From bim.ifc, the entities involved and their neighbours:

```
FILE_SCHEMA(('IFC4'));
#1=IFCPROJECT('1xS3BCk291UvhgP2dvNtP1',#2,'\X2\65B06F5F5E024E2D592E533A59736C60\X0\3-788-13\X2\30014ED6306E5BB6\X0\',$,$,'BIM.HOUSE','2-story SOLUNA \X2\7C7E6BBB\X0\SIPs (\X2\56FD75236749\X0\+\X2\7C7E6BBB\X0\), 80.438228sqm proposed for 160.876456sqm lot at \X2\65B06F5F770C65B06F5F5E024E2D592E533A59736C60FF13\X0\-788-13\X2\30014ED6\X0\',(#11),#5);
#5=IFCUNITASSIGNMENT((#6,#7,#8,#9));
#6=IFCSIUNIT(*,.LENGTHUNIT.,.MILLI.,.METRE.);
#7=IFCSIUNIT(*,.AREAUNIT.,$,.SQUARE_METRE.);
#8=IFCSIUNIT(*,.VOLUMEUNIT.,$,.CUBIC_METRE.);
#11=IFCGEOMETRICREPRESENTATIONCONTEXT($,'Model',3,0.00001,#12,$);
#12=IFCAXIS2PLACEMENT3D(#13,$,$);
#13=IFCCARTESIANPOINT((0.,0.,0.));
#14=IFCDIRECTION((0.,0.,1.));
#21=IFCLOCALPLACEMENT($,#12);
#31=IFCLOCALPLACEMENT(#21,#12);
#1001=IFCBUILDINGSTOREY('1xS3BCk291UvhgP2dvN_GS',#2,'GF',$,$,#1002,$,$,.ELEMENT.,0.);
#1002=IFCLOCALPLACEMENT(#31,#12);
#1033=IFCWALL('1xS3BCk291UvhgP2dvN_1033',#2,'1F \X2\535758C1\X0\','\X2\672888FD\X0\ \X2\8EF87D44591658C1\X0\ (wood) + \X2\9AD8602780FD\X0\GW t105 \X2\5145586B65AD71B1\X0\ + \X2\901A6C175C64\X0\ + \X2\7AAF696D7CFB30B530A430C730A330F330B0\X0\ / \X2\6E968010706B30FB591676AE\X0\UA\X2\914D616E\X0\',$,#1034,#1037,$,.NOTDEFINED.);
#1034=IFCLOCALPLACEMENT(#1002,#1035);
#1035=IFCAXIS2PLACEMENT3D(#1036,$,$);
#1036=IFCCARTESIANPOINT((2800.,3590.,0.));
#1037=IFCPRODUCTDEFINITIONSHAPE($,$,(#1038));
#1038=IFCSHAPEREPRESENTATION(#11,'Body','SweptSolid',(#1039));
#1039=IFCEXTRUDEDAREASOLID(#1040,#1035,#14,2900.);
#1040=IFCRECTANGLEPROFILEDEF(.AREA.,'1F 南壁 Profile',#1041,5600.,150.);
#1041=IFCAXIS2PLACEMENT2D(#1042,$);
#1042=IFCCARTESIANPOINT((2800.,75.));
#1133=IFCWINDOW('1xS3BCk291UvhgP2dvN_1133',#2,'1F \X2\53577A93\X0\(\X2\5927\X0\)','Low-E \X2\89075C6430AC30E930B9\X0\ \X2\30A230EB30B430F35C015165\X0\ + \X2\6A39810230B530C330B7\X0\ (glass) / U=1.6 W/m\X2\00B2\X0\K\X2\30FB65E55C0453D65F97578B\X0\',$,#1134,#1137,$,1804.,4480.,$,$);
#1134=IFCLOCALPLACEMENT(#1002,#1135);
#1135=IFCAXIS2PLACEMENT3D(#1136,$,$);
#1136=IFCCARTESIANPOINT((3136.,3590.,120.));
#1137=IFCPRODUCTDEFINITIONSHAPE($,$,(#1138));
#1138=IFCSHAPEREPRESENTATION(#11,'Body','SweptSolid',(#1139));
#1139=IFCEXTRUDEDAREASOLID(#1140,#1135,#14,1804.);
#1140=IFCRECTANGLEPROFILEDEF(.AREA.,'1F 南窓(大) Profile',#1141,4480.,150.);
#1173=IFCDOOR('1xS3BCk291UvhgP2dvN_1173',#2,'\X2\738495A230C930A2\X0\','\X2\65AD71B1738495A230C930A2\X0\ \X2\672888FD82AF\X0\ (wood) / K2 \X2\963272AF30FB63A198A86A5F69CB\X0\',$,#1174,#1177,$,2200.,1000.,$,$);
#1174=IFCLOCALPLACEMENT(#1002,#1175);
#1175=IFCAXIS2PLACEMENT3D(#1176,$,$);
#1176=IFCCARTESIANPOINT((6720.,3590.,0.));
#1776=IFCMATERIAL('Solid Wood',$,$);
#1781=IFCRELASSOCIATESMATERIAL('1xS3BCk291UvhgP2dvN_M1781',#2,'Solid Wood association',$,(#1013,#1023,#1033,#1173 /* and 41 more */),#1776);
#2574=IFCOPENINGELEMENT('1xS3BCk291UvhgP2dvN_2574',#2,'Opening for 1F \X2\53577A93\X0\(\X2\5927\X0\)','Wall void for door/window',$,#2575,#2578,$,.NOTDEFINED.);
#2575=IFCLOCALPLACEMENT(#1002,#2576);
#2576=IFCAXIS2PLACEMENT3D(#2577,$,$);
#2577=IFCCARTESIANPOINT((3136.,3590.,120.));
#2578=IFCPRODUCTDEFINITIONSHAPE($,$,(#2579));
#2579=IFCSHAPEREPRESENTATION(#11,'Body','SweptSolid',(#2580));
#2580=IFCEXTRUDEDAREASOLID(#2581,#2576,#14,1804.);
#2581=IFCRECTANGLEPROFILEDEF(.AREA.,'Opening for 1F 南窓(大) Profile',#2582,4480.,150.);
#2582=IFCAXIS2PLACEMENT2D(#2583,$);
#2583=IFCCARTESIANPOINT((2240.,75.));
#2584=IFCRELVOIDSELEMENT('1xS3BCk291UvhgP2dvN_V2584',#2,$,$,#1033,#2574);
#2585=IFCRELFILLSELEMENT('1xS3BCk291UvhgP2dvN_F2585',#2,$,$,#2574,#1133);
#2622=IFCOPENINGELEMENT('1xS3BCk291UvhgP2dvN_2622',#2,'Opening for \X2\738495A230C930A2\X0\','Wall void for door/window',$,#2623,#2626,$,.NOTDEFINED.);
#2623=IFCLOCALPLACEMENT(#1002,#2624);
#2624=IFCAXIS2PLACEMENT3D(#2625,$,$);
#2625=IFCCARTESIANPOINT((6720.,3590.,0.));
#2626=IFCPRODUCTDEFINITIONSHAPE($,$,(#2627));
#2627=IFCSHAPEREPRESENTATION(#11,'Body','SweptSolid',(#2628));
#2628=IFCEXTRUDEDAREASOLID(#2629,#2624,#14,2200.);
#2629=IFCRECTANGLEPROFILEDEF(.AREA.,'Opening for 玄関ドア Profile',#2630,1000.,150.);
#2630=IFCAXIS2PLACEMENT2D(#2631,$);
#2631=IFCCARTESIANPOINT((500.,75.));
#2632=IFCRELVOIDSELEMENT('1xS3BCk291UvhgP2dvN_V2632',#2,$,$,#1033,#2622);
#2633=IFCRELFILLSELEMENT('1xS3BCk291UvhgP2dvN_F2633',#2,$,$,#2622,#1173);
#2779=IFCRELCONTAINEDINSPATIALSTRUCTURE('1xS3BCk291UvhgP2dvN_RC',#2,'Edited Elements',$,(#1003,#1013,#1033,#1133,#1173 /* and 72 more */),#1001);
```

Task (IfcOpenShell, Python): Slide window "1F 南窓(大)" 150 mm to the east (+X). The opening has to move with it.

```python
import ifcopenshell
import ifcopenshell.api.geometry
import ifcopenshell.util.placement
import ifcopenshell.util.unit

model = ifcopenshell.open("bim.ifc")
unit_scale = ifcopenshell.util.unit.calculate_unit_scale(model)

window = model.by_guid("1xS3BCk291UvhgP2dvN_1133")
opening = window.FillsVoids[0].RelatingOpeningElement
wall = opening.VoidsElements[0].RelatingBuildingElement

wall_matrix = ifcopenshell.util.placement.get_local_placement(wall.ObjectPlacement)
shift = wall_matrix[:3, 0] * 0.15 / unit_scale
before = ifcopenshell.util.placement.get_local_placement(window.ObjectPlacement)[:3, 3].copy()

# The window is not placed relative to its opening, so move both.
for product in (opening, window):
    matrix = ifcopenshell.util.placement.get_local_placement(product.ObjectPlacement)
    matrix[:3, 3] += shift
    ifcopenshell.api.geometry.edit_object_placement(model, product=product, matrix=matrix, is_si=False)

after = ifcopenshell.util.placement.get_local_placement(window.ObjectPlacement)[:3, 3]
print("window moved by", (after - before).round(3) + 0.0)

model.write("bim_updated.ifc")
```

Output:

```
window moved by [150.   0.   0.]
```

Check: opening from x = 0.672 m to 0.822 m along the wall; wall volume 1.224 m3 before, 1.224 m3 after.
